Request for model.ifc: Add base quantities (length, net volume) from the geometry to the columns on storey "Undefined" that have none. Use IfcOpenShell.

First a look at what the model holds.

```python
import ifcopenshell
import ifcopenshell.util.element
import ifcopenshell.util.unit

model = ifcopenshell.open("model.ifc")
print(model.schema)
for unit_type in ("LENGTHUNIT", "AREAUNIT", "VOLUMEUNIT"):
    print(unit_type, ifcopenshell.util.unit.calculate_unit_scale(model, unit_type))
storey = next(s for s in model.by_type("IfcBuildingStorey") if s.Name == "Undefined")
columns = [e for e in ifcopenshell.util.element.get_decomposition(storey) if e.is_a("IfcColumn")]
for e in sorted(columns, key=lambda e: e.id()):
    print(e.id(), e.is_a(), e.Name, list(ifcopenshell.util.element.get_psets(e, qtos_only=True)), sep=" | ")
```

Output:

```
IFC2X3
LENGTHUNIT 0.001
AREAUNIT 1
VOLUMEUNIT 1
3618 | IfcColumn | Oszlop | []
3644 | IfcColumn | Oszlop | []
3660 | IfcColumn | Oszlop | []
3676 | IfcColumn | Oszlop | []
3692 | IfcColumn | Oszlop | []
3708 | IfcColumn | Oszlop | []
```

```python
import ifcopenshell
import ifcopenshell.api.pset
import ifcopenshell.geom
import ifcopenshell.util.element
import ifcopenshell.util.shape
import ifcopenshell.util.unit

model = ifcopenshell.open("model.ifc")
unit_scale = ifcopenshell.util.unit.calculate_unit_scale(model)
volume_scale = ifcopenshell.util.unit.calculate_unit_scale(model, "VOLUMEUNIT")
settings = ifcopenshell.geom.settings()

storey = next(s for s in model.by_type("IfcBuildingStorey") if s.Name == "Undefined")
columns = [e for e in ifcopenshell.util.element.get_decomposition(storey) if e.is_a("IfcColumn")]

for e in sorted(columns, key=lambda e: e.id()):
    if ifcopenshell.util.element.get_psets(e, qtos_only=True, should_inherit=False):
        continue
    # Geometry comes back in metres, in the element's own axes.
    shape = ifcopenshell.geom.create_shape(settings, e)
    values = {
        "Length": ifcopenshell.util.shape.get_z(shape.geometry) / unit_scale,
        "NetVolume": ifcopenshell.util.shape.get_volume(shape.geometry) / volume_scale,
    }
    qto = ifcopenshell.api.pset.add_qto(model, product=e, name="BaseQuantities")
    ifcopenshell.api.pset.edit_qto(model, qto=qto, properties=values)
    print(e.id(), {k: round(v, 3) for k, v in values.items()})

model.write("model_updated.ifc")
```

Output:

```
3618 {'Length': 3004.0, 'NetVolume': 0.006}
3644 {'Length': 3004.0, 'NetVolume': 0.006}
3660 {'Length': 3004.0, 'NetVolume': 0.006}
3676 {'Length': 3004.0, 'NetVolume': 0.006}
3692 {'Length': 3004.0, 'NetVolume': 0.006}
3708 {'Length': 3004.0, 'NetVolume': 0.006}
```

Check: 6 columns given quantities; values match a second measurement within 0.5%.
